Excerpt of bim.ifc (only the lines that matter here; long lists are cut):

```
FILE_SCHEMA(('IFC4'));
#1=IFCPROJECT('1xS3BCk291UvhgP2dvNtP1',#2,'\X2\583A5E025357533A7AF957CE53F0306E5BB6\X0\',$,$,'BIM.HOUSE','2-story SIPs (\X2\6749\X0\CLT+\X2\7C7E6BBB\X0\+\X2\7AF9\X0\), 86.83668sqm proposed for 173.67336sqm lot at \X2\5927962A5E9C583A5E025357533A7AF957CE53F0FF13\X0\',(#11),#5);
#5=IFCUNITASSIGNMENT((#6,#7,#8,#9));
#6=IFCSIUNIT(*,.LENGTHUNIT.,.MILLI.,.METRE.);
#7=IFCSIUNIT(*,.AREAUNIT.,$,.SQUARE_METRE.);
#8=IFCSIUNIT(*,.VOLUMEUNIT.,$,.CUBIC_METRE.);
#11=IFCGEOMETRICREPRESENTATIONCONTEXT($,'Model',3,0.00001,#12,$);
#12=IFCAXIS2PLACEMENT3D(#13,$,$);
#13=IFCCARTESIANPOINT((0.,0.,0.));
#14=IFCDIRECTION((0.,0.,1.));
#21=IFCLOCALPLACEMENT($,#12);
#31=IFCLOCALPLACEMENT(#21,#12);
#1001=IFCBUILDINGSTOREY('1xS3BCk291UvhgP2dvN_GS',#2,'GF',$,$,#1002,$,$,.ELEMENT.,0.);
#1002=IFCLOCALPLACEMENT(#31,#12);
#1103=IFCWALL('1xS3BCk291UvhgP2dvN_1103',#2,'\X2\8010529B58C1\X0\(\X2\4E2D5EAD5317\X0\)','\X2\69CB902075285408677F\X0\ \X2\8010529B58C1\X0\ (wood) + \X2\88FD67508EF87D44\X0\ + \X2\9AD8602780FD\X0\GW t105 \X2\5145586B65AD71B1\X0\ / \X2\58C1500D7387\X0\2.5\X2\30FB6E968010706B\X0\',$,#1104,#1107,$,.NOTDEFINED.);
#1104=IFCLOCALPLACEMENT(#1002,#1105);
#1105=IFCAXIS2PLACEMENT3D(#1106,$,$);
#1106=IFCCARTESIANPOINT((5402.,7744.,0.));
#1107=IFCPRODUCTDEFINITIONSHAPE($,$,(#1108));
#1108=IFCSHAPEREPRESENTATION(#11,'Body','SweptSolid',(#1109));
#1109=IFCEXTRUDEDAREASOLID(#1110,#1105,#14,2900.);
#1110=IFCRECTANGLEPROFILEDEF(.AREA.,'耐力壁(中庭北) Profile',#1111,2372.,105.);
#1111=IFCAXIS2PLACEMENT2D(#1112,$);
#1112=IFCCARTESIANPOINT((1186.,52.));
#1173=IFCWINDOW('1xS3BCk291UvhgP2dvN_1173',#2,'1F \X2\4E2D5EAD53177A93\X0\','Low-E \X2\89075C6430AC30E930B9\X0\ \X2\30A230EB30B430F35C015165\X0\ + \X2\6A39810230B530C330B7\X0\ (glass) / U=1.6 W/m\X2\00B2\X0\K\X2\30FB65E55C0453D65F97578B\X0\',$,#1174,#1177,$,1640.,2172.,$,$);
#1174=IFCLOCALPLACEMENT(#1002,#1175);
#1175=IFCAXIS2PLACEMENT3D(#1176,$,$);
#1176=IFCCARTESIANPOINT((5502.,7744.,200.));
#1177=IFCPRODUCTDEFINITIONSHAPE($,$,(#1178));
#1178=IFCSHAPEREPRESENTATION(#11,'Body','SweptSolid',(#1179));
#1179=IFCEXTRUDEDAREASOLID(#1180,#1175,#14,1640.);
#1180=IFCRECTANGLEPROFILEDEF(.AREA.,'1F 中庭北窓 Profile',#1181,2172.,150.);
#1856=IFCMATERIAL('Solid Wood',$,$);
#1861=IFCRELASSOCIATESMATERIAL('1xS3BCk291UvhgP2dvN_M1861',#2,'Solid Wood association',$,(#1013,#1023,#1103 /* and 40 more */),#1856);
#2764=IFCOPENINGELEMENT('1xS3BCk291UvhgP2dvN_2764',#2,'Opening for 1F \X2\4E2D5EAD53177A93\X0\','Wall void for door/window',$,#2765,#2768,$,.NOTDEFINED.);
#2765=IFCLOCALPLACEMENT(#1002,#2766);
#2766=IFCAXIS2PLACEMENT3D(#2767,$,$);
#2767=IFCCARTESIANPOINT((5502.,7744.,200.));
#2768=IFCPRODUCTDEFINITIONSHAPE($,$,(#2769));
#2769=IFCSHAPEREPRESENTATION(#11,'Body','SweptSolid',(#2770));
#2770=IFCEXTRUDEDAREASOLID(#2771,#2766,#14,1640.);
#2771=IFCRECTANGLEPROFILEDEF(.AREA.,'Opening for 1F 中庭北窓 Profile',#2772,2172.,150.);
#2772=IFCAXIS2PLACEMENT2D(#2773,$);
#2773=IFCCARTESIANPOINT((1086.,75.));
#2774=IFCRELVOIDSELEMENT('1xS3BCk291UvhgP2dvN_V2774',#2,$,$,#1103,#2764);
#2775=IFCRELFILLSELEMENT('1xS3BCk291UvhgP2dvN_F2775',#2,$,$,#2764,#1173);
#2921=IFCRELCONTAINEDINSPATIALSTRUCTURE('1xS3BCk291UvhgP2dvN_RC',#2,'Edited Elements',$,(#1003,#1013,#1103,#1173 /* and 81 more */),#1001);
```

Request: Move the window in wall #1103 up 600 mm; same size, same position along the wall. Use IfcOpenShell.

```python
import numpy as np
import ifcopenshell
import ifcopenshell.api.geometry
import ifcopenshell.util.placement
import ifcopenshell.util.unit

model = ifcopenshell.open("bim.ifc")
unit_scale = ifcopenshell.util.unit.calculate_unit_scale(model)

window = model.by_id(1173)
opening = window.FillsVoids[0].RelatingOpeningElement
dz = 0.6 / unit_scale

shift = np.array([0.0, 0.0, dz])
# The window is not placed relative to its opening, so move both.
for product in (opening, window):
    matrix = ifcopenshell.util.placement.get_local_placement(product.ObjectPlacement)
    matrix[:3, 3] += shift
    ifcopenshell.api.geometry.edit_object_placement(model, product=product, matrix=matrix, is_si=False)

print(f"moved by {dz * unit_scale:+.3f} m")

model.write("bim_updated.ifc")
```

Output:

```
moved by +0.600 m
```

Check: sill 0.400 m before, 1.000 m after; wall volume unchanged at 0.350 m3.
